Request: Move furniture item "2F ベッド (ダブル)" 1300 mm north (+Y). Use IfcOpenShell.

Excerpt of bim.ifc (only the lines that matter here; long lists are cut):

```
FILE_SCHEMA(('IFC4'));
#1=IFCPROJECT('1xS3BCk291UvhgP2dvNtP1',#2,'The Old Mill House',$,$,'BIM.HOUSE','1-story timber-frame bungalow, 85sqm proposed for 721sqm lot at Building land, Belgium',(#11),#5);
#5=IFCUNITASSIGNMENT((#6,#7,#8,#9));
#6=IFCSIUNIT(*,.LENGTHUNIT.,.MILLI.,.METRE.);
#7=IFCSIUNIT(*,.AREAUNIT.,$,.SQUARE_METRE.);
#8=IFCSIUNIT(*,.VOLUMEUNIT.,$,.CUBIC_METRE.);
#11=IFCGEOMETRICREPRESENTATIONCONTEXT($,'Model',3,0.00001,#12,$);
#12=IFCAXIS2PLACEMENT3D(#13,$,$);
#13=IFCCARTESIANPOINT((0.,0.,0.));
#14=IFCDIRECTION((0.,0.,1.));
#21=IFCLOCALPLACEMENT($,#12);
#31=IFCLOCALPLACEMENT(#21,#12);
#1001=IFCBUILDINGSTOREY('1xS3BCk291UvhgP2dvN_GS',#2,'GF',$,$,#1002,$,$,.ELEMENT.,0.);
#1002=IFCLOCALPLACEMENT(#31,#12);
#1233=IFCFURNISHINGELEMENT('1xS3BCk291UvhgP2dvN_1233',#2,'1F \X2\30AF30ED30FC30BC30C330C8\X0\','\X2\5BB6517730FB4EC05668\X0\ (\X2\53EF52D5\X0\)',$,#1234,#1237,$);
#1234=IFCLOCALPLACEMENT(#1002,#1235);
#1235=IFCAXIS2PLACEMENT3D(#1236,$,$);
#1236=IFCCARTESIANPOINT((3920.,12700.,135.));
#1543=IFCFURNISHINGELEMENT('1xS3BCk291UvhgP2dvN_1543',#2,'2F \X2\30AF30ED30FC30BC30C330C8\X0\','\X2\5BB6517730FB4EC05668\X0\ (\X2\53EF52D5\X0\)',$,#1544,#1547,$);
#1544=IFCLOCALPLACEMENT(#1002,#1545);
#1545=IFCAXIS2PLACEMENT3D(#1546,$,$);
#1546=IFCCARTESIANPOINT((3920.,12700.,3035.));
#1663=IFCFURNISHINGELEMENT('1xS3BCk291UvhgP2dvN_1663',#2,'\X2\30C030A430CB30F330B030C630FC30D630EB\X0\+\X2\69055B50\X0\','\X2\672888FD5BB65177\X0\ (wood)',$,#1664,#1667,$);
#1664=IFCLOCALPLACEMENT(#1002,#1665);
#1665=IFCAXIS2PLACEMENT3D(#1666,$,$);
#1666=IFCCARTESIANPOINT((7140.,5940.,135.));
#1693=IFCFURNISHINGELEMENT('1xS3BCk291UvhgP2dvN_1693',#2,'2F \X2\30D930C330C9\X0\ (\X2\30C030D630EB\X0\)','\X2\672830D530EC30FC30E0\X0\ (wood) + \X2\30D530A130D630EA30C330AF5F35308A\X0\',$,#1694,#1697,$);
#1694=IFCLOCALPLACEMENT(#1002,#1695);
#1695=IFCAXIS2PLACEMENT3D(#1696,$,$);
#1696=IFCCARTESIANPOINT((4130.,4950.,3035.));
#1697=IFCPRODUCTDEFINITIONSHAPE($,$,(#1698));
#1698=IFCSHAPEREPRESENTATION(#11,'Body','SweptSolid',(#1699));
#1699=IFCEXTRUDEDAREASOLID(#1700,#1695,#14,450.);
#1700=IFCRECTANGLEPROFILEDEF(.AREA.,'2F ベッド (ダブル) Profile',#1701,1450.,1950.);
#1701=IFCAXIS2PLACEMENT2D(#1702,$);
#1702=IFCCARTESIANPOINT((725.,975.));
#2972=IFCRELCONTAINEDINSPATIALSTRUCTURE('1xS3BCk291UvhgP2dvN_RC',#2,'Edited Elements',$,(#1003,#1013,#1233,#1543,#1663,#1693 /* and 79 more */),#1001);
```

```python
import ifcopenshell
import ifcopenshell.api.geometry
import ifcopenshell.util.placement
import ifcopenshell.util.unit

model = ifcopenshell.open("bim.ifc")
unit_scale = ifcopenshell.util.unit.calculate_unit_scale(model)

item = model.by_guid("1xS3BCk291UvhgP2dvN_1693")
matrix = ifcopenshell.util.placement.get_local_placement(item.ObjectPlacement)
matrix[1, 3] += 1.3 / unit_scale
ifcopenshell.api.geometry.edit_object_placement(model, product=item, matrix=matrix, is_si=False)

print(ifcopenshell.util.placement.get_local_placement(item.ObjectPlacement).round(3) + 0.0)

model.write("bim_edited.ifc")
```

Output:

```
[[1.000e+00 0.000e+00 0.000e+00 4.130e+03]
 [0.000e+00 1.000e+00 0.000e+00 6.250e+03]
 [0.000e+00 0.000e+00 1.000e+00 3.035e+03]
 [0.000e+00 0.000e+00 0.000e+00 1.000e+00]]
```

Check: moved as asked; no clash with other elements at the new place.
